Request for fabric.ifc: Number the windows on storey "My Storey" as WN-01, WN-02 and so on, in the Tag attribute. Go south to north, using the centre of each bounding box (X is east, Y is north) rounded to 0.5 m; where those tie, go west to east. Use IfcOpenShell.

First a look at what the model holds.

```python
import ifcopenshell
import ifcopenshell.util.element
import ifcopenshell.util.placement

model = ifcopenshell.open("fabric.ifc")
print(model.schema)
storey = next(s for s in model.by_type("IfcBuildingStorey") if s.Name == "My Storey")
windows = [e for e in ifcopenshell.util.element.get_decomposition(storey) if e.is_a("IfcWindow")]
for e in sorted(windows, key=lambda e: e.id()):
    origin = ifcopenshell.util.placement.get_local_placement(e.ObjectPlacement)[:3, 3]
    print(e.id(), e.Tag, e.Name, origin.round(2) + 0.0, sep=" | ")
```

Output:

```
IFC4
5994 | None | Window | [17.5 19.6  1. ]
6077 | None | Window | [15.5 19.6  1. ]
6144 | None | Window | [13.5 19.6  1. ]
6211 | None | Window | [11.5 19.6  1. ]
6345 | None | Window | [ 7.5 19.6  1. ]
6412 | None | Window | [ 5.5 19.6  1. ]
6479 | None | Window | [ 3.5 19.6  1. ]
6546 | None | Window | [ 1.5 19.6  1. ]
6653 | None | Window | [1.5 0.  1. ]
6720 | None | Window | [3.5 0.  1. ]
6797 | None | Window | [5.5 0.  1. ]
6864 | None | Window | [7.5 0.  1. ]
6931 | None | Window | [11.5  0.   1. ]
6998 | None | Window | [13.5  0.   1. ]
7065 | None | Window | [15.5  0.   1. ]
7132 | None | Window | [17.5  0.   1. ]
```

```python
import ifcopenshell
import ifcopenshell.geom
import ifcopenshell.util.element
import ifcopenshell.util.shape

model = ifcopenshell.open("fabric.ifc")
settings = ifcopenshell.geom.settings()
settings.set("use-world-coords", True)


def centre(element):
    shape = ifcopenshell.geom.create_shape(settings, element)
    return ifcopenshell.util.shape.get_bbox_centroid(shape.geometry)


storey = next(s for s in model.by_type("IfcBuildingStorey") if s.Name == "My Storey")
windows = [e for e in ifcopenshell.util.element.get_decomposition(storey) if e.is_a("IfcWindow")]

# Insertion points can sit at a corner or the storey origin, so sort by the geometry (in metres).
centres = {e: centre(e) for e in windows}
windows.sort(key=lambda e: (round(centres[e][1] / 0.5), centres[e][0]))

for i, e in enumerate(windows, start=1):
    number = f"WN-{i:02d}"
    e.Tag = number
    print(e.id(), number)

model.write("fabric_edited.ifc")
```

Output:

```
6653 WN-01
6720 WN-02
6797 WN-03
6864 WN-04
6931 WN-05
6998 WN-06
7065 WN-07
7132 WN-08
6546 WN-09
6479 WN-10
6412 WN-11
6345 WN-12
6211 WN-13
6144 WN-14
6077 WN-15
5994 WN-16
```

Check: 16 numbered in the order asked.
